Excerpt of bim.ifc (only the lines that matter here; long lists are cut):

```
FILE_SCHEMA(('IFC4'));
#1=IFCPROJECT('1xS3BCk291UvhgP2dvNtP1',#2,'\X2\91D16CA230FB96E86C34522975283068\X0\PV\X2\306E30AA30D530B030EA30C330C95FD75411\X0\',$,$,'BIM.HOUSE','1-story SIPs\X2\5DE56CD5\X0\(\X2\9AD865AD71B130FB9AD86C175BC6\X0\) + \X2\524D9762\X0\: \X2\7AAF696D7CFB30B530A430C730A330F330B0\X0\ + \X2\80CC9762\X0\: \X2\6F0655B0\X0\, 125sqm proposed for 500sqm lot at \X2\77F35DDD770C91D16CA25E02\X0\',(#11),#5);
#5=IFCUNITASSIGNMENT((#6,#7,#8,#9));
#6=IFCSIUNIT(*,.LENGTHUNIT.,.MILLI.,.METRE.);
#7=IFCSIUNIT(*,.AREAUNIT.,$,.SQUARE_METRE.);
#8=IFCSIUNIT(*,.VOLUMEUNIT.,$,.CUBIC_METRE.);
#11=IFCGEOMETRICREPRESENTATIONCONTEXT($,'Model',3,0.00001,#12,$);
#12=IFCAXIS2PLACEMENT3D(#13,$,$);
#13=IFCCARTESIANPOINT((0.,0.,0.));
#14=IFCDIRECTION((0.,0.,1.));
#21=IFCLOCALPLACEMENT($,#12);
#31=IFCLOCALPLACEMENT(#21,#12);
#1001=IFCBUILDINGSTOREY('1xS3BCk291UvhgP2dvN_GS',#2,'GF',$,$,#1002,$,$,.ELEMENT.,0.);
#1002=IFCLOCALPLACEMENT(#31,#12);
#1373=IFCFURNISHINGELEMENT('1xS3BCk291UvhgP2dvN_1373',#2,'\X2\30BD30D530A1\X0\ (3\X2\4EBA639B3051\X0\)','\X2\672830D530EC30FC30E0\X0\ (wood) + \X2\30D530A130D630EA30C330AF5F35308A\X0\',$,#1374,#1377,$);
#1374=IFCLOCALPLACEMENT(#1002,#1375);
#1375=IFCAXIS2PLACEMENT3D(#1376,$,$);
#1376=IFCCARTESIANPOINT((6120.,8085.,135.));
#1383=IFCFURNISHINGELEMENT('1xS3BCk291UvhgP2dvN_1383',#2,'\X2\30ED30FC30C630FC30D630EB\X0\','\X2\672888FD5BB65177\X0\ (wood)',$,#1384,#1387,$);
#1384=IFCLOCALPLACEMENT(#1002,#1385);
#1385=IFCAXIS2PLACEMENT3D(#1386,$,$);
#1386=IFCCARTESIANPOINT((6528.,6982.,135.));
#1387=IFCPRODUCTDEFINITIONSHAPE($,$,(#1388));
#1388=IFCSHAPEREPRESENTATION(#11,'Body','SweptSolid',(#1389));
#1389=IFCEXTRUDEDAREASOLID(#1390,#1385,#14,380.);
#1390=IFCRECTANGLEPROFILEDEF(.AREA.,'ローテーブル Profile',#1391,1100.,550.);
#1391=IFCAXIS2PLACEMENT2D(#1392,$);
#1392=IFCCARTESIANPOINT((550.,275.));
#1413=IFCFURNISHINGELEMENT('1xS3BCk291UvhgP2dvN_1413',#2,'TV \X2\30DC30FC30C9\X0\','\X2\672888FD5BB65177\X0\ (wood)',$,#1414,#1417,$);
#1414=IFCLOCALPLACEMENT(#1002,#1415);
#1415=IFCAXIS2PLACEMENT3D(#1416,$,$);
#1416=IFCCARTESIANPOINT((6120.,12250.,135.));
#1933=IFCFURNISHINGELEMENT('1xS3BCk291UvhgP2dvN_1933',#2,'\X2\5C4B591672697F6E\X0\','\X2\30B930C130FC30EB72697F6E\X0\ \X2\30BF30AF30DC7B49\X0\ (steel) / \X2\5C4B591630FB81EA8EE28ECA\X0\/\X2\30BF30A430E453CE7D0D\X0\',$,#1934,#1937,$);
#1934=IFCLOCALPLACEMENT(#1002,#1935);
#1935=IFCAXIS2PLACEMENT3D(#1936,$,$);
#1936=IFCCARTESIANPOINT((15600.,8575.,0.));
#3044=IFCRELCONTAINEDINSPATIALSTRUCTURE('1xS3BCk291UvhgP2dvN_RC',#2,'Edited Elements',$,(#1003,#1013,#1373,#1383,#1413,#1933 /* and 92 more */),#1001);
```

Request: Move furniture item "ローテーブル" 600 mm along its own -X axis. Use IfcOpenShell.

```python
import ifcopenshell
import ifcopenshell.api.geometry
import ifcopenshell.util.placement
import ifcopenshell.util.unit

model = ifcopenshell.open("bim.ifc")
unit_scale = ifcopenshell.util.unit.calculate_unit_scale(model)

item = model.by_guid("1xS3BCk291UvhgP2dvN_1383")
matrix = ifcopenshell.util.placement.get_local_placement(item.ObjectPlacement)
matrix[:3, 3] -= matrix[:3, 0] * 0.6 / unit_scale
ifcopenshell.api.geometry.edit_object_placement(model, product=item, matrix=matrix, is_si=False)

print(ifcopenshell.util.placement.get_local_placement(item.ObjectPlacement).round(3) + 0.0)

model.write("bim_updated.ifc")
```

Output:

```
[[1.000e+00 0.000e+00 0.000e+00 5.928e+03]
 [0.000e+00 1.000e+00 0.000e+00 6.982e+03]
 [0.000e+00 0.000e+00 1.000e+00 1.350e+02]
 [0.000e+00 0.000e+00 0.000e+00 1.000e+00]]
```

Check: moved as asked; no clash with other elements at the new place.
